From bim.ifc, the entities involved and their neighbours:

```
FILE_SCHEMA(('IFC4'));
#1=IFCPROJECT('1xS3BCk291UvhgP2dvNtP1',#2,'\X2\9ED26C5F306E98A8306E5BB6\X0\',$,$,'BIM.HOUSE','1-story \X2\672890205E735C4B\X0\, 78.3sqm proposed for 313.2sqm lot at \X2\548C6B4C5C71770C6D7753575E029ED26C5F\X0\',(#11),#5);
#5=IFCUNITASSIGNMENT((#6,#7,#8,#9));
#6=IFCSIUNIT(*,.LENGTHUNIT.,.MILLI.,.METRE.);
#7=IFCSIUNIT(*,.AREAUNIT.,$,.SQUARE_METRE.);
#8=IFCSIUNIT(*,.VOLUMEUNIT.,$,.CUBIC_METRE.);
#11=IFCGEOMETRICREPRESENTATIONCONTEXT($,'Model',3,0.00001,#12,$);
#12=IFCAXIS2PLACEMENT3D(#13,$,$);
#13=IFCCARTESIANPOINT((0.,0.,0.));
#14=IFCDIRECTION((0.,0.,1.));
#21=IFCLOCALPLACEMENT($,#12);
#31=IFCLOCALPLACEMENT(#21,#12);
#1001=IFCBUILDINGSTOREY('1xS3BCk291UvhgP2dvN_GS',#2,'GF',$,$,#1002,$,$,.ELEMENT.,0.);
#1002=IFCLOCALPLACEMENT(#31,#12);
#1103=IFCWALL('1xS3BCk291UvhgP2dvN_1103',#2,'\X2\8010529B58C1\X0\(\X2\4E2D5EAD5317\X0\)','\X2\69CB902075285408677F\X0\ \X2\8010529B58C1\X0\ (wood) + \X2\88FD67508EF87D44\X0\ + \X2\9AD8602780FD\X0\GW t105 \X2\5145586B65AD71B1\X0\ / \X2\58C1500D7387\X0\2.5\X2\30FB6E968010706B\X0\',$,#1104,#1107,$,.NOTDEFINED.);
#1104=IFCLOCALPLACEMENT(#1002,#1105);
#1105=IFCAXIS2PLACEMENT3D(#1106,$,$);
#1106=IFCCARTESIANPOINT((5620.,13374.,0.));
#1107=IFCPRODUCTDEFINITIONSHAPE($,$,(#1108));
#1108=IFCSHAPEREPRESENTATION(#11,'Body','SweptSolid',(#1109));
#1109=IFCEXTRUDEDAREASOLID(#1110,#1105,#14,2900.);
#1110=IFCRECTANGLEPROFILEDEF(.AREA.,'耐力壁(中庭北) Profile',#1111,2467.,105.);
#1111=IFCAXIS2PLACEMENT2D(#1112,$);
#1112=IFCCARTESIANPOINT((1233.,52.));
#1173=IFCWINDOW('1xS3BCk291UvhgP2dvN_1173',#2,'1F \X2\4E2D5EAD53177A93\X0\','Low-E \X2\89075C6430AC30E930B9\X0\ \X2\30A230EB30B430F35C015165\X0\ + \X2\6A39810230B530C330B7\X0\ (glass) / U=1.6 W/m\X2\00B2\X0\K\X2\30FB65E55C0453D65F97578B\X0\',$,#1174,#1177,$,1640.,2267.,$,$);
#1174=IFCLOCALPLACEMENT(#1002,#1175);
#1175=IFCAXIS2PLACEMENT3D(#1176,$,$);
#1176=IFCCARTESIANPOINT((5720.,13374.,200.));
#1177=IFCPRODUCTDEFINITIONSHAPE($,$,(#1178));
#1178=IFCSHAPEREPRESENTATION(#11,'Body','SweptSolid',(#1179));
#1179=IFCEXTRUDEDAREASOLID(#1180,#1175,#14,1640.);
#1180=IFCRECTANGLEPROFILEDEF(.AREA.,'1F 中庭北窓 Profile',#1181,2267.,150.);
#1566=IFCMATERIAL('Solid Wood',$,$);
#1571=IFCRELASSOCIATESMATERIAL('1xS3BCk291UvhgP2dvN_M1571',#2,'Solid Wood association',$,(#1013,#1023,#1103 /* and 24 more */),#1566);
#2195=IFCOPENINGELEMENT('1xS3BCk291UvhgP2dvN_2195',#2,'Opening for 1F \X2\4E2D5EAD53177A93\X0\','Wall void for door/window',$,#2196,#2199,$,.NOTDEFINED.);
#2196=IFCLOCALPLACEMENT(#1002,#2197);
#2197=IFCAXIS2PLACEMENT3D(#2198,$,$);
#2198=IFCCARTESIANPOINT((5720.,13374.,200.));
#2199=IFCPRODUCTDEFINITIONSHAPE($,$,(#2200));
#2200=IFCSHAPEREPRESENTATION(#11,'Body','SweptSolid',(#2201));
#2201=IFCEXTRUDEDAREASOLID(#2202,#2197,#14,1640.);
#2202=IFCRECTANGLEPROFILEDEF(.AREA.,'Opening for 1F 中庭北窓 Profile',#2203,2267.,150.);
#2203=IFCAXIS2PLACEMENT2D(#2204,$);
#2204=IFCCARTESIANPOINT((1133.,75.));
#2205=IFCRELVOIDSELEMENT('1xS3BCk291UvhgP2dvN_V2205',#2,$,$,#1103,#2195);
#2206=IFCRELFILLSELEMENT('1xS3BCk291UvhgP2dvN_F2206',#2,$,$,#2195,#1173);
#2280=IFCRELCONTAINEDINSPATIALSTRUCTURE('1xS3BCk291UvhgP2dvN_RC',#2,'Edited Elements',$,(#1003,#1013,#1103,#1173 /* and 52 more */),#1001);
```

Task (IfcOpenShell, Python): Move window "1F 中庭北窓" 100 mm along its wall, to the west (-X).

```python
import ifcopenshell
import ifcopenshell.api.geometry
import ifcopenshell.util.placement
import ifcopenshell.util.unit

model = ifcopenshell.open("bim.ifc")
unit_scale = ifcopenshell.util.unit.calculate_unit_scale(model)

window = model.by_guid("1xS3BCk291UvhgP2dvN_1173")
opening = window.FillsVoids[0].RelatingOpeningElement
wall = opening.VoidsElements[0].RelatingBuildingElement

wall_matrix = ifcopenshell.util.placement.get_local_placement(wall.ObjectPlacement)
shift = wall_matrix[:3, 0] * -0.1 / unit_scale
before = ifcopenshell.util.placement.get_local_placement(window.ObjectPlacement)[:3, 3].copy()

# The window is not placed relative to its opening, so move both.
for product in (opening, window):
    matrix = ifcopenshell.util.placement.get_local_placement(product.ObjectPlacement)
    matrix[:3, 3] += shift
    ifcopenshell.api.geometry.edit_object_placement(model, product=product, matrix=matrix, is_si=False)

after = ifcopenshell.util.placement.get_local_placement(window.ObjectPlacement)[:3, 3]
print("window moved by", (after - before).round(3) + 0.0)

model.write("bim_rev.ifc")
```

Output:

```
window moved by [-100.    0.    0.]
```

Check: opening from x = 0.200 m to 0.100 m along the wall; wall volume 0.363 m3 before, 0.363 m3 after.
